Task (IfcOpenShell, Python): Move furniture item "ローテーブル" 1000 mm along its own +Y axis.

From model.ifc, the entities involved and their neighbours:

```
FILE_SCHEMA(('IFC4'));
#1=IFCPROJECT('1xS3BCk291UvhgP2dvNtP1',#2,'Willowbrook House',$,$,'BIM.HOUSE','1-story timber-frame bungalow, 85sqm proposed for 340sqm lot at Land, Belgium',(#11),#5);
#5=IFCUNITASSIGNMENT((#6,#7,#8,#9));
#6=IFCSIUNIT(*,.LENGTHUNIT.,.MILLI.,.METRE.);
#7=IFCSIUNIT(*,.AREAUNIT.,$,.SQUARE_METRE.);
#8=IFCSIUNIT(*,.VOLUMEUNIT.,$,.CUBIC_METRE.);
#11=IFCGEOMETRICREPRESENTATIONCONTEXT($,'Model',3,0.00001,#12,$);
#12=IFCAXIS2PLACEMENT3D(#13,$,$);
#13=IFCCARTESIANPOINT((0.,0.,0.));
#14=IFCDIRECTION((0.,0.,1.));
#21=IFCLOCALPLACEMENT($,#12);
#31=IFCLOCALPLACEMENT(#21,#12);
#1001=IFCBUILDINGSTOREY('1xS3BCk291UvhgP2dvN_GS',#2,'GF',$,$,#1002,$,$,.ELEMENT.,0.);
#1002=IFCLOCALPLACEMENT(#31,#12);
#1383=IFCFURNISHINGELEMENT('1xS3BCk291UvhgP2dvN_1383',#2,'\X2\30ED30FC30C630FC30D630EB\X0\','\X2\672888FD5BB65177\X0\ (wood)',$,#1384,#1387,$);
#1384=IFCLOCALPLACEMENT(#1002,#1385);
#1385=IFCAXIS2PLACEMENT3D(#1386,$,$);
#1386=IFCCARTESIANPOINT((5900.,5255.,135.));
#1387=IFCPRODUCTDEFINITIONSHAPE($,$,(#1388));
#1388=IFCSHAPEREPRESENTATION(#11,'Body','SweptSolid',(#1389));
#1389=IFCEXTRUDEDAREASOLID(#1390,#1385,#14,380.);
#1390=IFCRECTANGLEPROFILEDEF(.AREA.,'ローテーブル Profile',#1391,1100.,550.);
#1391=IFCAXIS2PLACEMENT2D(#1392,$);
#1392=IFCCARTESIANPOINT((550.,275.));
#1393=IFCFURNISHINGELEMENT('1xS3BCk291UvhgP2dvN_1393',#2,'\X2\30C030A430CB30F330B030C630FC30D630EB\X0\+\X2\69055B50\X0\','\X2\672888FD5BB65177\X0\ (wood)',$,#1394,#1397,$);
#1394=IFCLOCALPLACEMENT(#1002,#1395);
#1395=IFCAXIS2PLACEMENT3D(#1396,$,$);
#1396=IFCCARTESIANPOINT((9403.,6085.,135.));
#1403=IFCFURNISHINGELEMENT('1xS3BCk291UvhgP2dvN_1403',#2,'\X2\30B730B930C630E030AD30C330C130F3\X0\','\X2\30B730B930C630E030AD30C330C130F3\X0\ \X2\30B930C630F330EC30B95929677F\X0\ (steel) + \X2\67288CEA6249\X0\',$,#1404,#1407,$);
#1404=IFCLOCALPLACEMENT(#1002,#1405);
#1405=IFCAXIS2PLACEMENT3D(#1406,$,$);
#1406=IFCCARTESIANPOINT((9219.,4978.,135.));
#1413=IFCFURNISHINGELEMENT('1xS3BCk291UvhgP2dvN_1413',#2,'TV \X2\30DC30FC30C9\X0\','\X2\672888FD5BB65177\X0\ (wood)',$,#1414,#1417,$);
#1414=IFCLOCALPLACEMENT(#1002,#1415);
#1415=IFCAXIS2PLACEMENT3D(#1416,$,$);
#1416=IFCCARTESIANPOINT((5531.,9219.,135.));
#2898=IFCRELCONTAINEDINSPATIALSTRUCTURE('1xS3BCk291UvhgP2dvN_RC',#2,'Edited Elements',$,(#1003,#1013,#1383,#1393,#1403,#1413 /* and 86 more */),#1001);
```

```python
import ifcopenshell
import ifcopenshell.api.geometry
import ifcopenshell.util.placement

model = ifcopenshell.open("model.ifc")

item = model.by_guid("1xS3BCk291UvhgP2dvN_1383")
matrix = ifcopenshell.util.placement.get_local_placement(item.ObjectPlacement)
matrix[:3, 3] += matrix[:3, 1] * 1000.0
ifcopenshell.api.geometry.edit_object_placement(model, product=item, matrix=matrix, is_si=False)

print(ifcopenshell.util.placement.get_local_placement(item.ObjectPlacement).round(3) + 0.0)

model.write("model_v2.ifc")
```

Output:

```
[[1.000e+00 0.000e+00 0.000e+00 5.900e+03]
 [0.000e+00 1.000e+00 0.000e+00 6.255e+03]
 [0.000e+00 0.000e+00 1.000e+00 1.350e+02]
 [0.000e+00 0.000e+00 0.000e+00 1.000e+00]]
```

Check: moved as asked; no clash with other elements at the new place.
